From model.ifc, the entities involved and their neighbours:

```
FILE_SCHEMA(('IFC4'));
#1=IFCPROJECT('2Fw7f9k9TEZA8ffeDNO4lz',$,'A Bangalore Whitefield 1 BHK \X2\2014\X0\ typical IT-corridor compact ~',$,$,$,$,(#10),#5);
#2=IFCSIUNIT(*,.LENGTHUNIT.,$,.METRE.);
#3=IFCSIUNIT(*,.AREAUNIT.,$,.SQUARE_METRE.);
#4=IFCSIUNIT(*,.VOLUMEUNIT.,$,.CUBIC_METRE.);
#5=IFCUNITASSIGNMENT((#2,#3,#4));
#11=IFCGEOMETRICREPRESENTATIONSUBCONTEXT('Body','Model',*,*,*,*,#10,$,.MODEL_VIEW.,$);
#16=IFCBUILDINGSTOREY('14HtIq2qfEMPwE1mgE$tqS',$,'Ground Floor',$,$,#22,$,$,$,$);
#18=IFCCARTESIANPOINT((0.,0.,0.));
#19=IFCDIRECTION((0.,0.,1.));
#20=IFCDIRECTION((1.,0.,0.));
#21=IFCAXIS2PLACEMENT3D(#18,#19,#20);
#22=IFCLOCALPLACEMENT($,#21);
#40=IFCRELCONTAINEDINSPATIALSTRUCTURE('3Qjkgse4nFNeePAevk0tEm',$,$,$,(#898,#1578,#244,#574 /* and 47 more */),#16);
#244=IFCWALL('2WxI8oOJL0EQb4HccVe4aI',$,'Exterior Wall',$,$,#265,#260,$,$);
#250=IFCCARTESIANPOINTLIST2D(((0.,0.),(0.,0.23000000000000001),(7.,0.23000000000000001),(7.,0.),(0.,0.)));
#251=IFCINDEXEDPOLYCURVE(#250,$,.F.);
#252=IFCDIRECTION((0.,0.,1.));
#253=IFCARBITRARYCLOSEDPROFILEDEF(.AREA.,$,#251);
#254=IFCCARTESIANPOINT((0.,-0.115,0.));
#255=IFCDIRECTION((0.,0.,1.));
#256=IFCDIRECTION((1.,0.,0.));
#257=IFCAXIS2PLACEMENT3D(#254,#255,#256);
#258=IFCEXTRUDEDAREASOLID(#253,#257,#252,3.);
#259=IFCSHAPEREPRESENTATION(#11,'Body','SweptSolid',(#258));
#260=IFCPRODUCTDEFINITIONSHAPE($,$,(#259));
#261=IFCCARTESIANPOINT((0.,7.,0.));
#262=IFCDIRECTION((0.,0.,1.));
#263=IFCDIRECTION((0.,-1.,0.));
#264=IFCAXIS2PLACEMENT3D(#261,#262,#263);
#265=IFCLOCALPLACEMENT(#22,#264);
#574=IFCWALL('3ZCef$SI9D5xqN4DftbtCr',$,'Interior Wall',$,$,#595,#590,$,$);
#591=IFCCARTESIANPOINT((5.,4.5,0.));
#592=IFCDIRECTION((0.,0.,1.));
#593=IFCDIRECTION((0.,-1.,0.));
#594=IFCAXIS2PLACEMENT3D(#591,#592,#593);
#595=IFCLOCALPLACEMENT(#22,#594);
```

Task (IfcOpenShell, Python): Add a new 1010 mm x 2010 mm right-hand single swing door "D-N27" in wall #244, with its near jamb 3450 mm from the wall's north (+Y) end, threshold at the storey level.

```python
import numpy as np
import ifcopenshell
import ifcopenshell.api.feature
import ifcopenshell.api.geometry
import ifcopenshell.api.root
import ifcopenshell.api.spatial
import ifcopenshell.geom
import ifcopenshell.util.element
import ifcopenshell.util.placement
import ifcopenshell.util.representation
import ifcopenshell.util.shape
import ifcopenshell.util.unit

model = ifcopenshell.open("model.ifc")
unit_scale = ifcopenshell.util.unit.calculate_unit_scale(model)
settings = ifcopenshell.geom.settings()


def volume(element):
    """Net volume in cubic metres, openings subtracted."""
    shape = ifcopenshell.geom.create_shape(settings, element)
    return ifcopenshell.util.shape.get_volume(shape.geometry)


wall = model.by_guid("2WxI8oOJL0EQb4HccVe4aI")
storey = ifcopenshell.util.element.get_container(wall, ifc_class="IfcBuildingStorey")
context = ifcopenshell.util.representation.get_context(model, "Model", "Body", "MODEL_VIEW")
before = volume(wall)

width, height, from_end, sill = 1.01, 2.01, 3.45, 0.0  # metres

# The wall runs along its own X axis, and the end named is its -X end.
wall_shape = ifcopenshell.geom.create_shape(settings, wall)
x, y, z = ifcopenshell.util.shape.get_vertices(wall_shape.geometry).T
start = x.min() + from_end
face, thickness = float(y.min()), float(y.max() - y.min())
wall_matrix = ifcopenshell.util.placement.get_local_placement(wall.ObjectPlacement)
level = ifcopenshell.util.placement.get_local_placement(storey.ObjectPlacement)[2, 3]


def in_wall(x, y):
    """Placement at x, y metres in the wall's axes, at sill height."""
    matrix = wall_matrix.copy()
    matrix[:, 3] = wall_matrix @ np.array([x / unit_scale, y / unit_scale, 0.0, 1.0])
    matrix[2, 3] = level + sill / unit_scale
    return matrix


# Opening: a box that overshoots both wall faces by 50 mm.
opening = ifcopenshell.api.root.create_entity(model, ifc_class="IfcOpeningElement", predefined_type="OPENING")
box = ifcopenshell.api.geometry.add_wall_representation(
    model, context=context, length=width, height=height, thickness=thickness + 0.1
)
ifcopenshell.api.geometry.assign_representation(model, product=opening, representation=box)
ifcopenshell.api.geometry.edit_object_placement(model, product=opening, matrix=in_wall(start, face - 0.05), is_si=False)
ifcopenshell.api.feature.add_feature(model, feature=opening, element=wall)

door = ifcopenshell.api.root.create_entity(model, ifc_class="IfcDoor", name="D-N27", predefined_type="DOOR")
door.OverallWidth, door.OverallHeight = width / unit_scale, height / unit_scale
door.OperationType = "SINGLE_SWING_RIGHT"
body = ifcopenshell.api.geometry.add_door_representation(
    model,
    context=context,
    overall_width=door.OverallWidth,
    overall_height=door.OverallHeight,
    operation_type="SINGLE_SWING_RIGHT",
    lining_properties={"LiningDepth": thickness / unit_scale, "ThresholdDepth": thickness / unit_scale},
)
ifcopenshell.api.geometry.assign_representation(model, product=door, representation=body)
ifcopenshell.api.spatial.assign_container(model, products=[door], relating_structure=storey)
ifcopenshell.api.feature.add_filling(model, opening=opening, element=door)

# The lining spans the wall, so the door starts at the wall face.
ifcopenshell.api.geometry.edit_object_placement(model, product=door, matrix=in_wall(start, face), is_si=False)

after = volume(wall)

print(f"wall volume {before:.3f} -> {after:.3f} m3")

model.write("model_v2.ifc")
```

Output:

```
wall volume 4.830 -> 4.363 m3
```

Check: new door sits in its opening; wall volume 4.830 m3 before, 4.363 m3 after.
